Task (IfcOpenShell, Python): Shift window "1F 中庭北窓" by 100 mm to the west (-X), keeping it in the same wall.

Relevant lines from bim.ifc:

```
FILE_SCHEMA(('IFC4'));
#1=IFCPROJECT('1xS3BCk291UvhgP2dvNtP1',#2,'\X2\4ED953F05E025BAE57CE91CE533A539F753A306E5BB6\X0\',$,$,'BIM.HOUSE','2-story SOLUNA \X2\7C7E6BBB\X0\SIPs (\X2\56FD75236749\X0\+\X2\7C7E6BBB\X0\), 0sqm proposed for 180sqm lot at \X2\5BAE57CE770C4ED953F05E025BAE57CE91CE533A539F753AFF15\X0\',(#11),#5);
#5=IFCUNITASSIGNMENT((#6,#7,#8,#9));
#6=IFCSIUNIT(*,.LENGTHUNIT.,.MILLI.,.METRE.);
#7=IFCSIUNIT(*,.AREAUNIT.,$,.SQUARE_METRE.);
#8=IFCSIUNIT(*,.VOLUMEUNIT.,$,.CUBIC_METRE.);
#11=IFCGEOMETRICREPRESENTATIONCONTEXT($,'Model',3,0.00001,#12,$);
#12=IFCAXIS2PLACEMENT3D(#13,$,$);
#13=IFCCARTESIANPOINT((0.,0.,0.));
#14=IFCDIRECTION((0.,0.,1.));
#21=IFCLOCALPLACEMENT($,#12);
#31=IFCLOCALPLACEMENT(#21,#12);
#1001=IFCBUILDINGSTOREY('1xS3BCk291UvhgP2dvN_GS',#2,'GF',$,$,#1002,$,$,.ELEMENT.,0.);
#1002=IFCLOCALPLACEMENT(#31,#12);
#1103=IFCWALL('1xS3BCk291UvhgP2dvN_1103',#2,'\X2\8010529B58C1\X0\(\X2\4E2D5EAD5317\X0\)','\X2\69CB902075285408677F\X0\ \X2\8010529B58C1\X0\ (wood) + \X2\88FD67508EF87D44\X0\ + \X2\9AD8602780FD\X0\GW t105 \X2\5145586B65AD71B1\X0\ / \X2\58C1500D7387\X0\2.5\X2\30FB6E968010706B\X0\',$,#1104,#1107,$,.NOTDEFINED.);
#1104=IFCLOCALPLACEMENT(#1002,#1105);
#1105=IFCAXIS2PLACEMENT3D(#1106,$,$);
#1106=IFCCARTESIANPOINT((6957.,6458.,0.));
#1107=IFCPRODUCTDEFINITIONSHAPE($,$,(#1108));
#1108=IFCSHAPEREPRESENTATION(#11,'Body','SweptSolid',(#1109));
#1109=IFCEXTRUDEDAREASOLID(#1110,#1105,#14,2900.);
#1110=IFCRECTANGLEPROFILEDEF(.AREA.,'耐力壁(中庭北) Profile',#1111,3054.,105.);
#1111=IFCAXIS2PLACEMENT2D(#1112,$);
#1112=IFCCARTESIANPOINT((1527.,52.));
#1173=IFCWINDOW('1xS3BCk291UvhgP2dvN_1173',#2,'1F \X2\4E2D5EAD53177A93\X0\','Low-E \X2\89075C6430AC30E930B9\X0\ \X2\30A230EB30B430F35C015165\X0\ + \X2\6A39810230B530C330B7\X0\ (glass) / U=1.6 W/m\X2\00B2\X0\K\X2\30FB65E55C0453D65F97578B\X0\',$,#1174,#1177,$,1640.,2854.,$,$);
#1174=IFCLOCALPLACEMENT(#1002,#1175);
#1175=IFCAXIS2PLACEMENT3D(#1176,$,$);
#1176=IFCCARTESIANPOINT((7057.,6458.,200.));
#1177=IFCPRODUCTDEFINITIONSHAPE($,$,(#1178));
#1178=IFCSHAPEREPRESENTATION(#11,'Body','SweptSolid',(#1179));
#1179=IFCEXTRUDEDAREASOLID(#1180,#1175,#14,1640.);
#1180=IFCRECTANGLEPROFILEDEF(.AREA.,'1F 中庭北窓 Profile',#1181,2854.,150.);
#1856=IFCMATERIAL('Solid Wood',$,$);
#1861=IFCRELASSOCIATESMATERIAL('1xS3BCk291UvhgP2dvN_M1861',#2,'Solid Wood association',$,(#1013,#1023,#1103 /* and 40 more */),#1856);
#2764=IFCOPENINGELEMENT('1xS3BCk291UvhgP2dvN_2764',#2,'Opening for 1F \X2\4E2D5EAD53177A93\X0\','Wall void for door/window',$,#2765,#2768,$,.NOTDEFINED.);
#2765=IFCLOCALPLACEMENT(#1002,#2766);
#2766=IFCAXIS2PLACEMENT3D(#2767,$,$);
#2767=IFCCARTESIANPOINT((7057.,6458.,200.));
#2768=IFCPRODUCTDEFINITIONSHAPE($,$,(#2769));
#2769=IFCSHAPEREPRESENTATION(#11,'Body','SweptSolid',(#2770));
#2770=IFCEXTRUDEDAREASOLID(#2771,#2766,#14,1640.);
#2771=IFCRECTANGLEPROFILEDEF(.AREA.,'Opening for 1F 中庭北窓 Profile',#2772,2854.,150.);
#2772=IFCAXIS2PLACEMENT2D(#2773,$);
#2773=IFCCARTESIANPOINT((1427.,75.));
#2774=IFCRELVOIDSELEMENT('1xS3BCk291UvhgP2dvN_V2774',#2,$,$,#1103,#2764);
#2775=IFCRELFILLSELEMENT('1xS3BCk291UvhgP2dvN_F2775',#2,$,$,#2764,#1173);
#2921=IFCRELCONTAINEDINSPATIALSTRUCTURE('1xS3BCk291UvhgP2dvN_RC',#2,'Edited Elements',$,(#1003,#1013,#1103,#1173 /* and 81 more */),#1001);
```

```python
import ifcopenshell
import ifcopenshell.api.geometry
import ifcopenshell.util.placement

model = ifcopenshell.open("bim.ifc")

window = model.by_guid("1xS3BCk291UvhgP2dvN_1173")
opening = window.FillsVoids[0].RelatingOpeningElement
wall = opening.VoidsElements[0].RelatingBuildingElement

wall_matrix = ifcopenshell.util.placement.get_local_placement(wall.ObjectPlacement)
shift = wall_matrix[:3, 0] * -100.0
before = ifcopenshell.util.placement.get_local_placement(window.ObjectPlacement)[:3, 3].copy()

# The window is not placed relative to its opening, so move both.
for product in (opening, window):
    matrix = ifcopenshell.util.placement.get_local_placement(product.ObjectPlacement)
    matrix[:3, 3] += shift
    ifcopenshell.api.geometry.edit_object_placement(model, product=product, matrix=matrix, is_si=False)

after = ifcopenshell.util.placement.get_local_placement(window.ObjectPlacement)[:3, 3]
print("window moved by", (after - before).round(3) + 0.0)

model.write("bim_edited.ifc")
```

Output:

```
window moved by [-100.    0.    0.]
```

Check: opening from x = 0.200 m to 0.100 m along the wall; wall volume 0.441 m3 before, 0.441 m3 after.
